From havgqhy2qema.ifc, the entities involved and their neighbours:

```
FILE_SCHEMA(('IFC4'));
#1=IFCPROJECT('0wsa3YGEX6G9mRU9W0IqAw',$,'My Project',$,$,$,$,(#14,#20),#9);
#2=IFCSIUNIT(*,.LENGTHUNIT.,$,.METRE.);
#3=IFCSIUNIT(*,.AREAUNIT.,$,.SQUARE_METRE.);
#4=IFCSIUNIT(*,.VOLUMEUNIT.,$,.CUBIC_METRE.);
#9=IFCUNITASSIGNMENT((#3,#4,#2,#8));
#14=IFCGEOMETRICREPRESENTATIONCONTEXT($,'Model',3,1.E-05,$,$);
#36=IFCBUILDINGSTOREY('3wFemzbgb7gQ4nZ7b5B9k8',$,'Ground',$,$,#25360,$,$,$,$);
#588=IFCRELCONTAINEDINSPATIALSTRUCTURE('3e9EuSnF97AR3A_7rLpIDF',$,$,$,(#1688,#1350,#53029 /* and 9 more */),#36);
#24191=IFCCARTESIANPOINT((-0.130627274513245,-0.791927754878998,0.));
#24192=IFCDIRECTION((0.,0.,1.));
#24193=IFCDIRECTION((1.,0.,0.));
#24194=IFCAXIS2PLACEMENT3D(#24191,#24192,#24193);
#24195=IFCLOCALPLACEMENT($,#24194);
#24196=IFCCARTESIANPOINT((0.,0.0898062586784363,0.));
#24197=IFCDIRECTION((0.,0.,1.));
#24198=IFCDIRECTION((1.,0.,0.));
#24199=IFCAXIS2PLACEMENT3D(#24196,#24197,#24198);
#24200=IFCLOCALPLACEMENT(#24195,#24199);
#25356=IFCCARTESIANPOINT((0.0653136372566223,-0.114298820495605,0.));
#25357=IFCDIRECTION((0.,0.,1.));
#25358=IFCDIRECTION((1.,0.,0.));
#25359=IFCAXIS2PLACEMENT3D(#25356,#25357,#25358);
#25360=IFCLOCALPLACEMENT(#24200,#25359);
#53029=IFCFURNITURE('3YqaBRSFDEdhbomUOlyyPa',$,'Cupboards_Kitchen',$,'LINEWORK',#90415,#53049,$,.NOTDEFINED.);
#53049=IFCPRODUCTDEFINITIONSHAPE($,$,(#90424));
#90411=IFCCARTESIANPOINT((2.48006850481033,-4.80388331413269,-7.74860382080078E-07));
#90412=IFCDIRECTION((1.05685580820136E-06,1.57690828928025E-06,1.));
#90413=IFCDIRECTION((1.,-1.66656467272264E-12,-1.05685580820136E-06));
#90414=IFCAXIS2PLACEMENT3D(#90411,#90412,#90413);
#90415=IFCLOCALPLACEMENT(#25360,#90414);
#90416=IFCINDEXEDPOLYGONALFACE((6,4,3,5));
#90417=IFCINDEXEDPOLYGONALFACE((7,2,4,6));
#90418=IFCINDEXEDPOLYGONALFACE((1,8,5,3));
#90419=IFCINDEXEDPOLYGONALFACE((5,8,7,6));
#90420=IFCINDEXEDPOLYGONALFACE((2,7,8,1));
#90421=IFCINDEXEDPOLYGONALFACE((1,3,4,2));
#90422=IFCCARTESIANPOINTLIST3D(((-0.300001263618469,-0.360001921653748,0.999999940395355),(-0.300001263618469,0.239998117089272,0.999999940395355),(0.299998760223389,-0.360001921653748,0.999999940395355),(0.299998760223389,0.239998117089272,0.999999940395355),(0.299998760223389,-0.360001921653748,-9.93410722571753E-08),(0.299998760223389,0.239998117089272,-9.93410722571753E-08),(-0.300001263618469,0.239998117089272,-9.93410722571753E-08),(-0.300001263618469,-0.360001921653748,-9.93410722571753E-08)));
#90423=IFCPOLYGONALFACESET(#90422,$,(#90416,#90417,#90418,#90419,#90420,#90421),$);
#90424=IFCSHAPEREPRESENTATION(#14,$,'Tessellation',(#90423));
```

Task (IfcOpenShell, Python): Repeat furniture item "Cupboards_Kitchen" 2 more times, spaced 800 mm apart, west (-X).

```python
import numpy as np
import ifcopenshell
import ifcopenshell.api.geometry
import ifcopenshell.api.root
import ifcopenshell.util.element
import ifcopenshell.util.placement

model = ifcopenshell.open("havgqhy2qema.ifc")

source = model.by_guid("3YqaBRSFDEdhbomUOlyyPa")
base = ifcopenshell.util.placement.get_local_placement(source.ObjectPlacement)
step = np.array([-1.0, 0.0, 0.0]) * 0.8

for i in range(1, 3):
    copy = ifcopenshell.api.root.copy_class(model, product=source)
    copy.Representation = ifcopenshell.util.element.copy_deep(
        model, source.Representation, exclude=["IfcGeometricRepresentationContext", "IfcRepresentationMap"]
    )
    matrix = base.copy()
    matrix[:3, 3] += i * step
    print("added at", matrix[:3, 3].round(3) + 0.0)
    ifcopenshell.api.geometry.edit_object_placement(model, product=copy, matrix=matrix, is_si=False)

model.write("havgqhy2qema_updated.ifc")
```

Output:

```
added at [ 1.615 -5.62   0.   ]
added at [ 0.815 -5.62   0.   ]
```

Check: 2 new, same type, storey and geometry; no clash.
